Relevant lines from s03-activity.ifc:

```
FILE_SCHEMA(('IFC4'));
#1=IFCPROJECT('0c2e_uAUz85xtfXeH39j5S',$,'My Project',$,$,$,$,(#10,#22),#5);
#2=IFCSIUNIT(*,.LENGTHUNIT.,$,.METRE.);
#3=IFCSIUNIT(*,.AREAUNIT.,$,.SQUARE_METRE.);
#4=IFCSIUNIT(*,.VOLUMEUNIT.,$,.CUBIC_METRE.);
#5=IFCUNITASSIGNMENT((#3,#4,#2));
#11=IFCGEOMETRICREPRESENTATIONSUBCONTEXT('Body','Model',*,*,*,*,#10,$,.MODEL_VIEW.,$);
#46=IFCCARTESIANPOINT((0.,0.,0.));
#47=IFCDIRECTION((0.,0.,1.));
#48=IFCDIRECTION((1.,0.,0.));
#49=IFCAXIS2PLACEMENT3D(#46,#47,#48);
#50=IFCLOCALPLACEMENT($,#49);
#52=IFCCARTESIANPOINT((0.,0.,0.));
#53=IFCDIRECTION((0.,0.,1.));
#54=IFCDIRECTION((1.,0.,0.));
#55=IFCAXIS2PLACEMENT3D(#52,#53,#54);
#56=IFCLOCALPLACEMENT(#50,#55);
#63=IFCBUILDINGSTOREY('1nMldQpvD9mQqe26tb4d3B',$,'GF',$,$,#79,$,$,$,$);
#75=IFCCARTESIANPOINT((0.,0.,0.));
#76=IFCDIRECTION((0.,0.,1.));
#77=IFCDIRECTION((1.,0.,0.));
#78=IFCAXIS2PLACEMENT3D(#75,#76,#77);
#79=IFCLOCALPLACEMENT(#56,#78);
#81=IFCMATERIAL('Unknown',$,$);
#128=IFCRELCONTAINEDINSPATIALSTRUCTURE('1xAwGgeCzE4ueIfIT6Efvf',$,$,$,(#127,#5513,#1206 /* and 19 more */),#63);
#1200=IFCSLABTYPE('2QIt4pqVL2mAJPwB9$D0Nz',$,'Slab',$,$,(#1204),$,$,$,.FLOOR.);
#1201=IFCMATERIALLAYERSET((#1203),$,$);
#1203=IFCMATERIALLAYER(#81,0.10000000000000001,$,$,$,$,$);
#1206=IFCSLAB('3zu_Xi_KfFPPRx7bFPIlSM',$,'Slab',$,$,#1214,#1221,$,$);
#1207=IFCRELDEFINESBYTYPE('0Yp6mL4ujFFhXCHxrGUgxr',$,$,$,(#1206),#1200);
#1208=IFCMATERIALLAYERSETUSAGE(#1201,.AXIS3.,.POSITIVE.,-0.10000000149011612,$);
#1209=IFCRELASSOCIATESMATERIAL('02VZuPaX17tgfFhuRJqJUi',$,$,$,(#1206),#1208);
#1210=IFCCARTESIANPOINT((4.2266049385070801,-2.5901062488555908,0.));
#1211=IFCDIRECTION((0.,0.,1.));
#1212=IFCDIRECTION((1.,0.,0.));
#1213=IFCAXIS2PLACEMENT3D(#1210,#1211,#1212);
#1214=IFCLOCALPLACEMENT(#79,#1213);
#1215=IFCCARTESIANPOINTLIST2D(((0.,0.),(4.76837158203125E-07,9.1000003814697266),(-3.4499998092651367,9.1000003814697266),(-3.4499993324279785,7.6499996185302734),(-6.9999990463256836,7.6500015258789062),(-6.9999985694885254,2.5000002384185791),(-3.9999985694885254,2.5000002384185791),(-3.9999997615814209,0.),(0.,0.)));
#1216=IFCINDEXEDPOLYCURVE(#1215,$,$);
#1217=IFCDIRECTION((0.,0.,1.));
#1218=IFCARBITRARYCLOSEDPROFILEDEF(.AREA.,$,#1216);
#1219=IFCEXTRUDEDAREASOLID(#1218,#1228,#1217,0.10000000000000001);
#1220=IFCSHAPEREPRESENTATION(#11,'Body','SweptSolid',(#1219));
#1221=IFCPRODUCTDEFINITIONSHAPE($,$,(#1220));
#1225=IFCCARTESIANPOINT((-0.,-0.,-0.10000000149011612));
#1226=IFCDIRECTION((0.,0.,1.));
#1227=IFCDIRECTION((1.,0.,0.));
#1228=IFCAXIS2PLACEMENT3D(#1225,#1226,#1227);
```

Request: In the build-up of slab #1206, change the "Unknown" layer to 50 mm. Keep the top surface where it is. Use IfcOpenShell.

```python
import ifcopenshell
import ifcopenshell.util.element
import ifcopenshell.util.representation

model = ifcopenshell.open("s03-activity.ifc")

layer_set = model.by_id(1201)
layer = next(l for l in layer_set.MaterialLayers if l.Material and l.Material.Name == "Unknown")
change = 0.05 - layer.LayerThickness
layer.LayerThickness += change

# Geometry does not follow the layer set by itself.
slabs = [e for e in ifcopenshell.util.element.get_elements_by_material(model, layer_set) if e.is_a("IfcSlab")]
for slab in sorted(slabs, key=lambda e: e.id()):
    body = ifcopenshell.util.representation.get_representation(slab, "Model", "Body")
    solid = body.Items[0]
    old_depth = solid.Depth
    solid.Depth += change
    # Extruded upwards: lower the start of the extrusion so the top stays.
    x, y, z = solid.Position.Location.Coordinates
    solid.Position.Location = model.createIfcCartesianPoint((x, y, z - change))
    print(slab.id(), f"{old_depth:g} -> {solid.Depth:g}")

# The layers are counted up from the underside, which has moved.
for usage in {ifcopenshell.util.element.get_material(slab) for slab in slabs}:
    usage.OffsetFromReferenceLine -= change

model.write("s03-activity_edited.ifc")
```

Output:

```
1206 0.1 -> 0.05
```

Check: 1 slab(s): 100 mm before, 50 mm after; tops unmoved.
